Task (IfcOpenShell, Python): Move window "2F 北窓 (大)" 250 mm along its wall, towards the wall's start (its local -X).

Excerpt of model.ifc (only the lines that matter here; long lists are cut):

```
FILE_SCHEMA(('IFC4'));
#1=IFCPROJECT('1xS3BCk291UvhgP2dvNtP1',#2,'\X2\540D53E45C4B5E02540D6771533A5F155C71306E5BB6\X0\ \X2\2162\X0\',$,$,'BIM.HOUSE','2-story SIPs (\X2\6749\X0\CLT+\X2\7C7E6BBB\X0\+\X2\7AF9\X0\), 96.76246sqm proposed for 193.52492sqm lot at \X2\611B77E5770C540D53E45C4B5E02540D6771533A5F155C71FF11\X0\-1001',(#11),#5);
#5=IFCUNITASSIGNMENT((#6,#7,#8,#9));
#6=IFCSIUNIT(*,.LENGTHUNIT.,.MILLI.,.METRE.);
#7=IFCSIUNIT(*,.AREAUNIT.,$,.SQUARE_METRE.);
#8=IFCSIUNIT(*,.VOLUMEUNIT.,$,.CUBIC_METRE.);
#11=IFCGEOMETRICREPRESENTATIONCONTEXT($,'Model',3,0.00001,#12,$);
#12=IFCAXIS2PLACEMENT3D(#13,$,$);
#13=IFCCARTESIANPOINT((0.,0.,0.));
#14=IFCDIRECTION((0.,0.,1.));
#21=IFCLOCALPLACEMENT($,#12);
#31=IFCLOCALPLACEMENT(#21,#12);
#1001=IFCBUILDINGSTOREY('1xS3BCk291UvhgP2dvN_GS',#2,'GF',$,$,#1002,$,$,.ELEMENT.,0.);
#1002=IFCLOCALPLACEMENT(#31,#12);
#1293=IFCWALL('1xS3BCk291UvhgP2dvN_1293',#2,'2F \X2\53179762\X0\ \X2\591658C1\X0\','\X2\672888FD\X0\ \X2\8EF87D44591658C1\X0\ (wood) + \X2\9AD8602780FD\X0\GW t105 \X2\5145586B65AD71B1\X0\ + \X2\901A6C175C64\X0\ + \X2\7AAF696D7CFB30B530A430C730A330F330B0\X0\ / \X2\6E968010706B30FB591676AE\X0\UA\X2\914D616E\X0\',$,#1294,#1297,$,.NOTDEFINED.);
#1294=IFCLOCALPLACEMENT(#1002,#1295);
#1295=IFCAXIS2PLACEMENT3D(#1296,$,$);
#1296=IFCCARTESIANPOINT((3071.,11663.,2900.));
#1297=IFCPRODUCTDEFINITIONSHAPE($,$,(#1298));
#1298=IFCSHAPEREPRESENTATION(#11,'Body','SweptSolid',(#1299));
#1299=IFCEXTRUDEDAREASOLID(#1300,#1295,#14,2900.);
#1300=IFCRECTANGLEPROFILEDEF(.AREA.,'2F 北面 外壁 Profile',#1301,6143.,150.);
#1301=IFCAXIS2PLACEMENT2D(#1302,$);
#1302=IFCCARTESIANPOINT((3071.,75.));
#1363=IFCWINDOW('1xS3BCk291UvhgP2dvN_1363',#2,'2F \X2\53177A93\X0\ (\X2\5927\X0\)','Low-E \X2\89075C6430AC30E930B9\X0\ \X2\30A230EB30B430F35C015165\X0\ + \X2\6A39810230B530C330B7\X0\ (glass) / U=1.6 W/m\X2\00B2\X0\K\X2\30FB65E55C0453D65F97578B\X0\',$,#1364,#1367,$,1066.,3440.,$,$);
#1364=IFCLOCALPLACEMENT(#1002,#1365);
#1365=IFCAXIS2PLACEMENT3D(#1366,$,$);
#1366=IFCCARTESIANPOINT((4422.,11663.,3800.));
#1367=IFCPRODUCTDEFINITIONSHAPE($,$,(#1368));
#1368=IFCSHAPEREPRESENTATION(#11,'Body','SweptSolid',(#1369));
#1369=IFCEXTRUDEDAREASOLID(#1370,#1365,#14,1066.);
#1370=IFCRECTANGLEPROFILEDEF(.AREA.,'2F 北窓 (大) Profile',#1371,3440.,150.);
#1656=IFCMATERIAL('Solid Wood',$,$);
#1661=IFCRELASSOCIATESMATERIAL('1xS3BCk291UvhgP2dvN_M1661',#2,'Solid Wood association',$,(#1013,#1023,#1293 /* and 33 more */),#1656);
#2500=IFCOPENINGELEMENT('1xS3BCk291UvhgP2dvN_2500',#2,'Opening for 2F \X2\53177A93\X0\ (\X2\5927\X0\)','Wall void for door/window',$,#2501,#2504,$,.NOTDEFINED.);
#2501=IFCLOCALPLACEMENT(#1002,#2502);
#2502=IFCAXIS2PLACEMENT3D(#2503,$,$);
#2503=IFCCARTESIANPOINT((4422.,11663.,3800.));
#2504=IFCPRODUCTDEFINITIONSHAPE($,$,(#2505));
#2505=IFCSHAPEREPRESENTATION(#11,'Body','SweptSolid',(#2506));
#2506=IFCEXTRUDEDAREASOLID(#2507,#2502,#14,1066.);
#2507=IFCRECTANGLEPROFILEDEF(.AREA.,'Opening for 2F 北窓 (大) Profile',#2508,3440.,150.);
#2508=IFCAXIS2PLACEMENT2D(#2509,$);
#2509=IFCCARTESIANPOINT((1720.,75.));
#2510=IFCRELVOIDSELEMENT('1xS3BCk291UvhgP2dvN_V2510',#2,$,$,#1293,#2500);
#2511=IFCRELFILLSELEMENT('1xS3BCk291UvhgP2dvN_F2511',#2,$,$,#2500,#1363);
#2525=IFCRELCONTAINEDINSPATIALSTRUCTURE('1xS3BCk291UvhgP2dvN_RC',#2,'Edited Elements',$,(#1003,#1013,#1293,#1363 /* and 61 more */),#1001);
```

```python
import ifcopenshell
import ifcopenshell.api.geometry
import ifcopenshell.util.placement
import ifcopenshell.util.unit

model = ifcopenshell.open("model.ifc")
unit_scale = ifcopenshell.util.unit.calculate_unit_scale(model)

window = model.by_guid("1xS3BCk291UvhgP2dvN_1363")
opening = window.FillsVoids[0].RelatingOpeningElement
wall = opening.VoidsElements[0].RelatingBuildingElement

wall_matrix = ifcopenshell.util.placement.get_local_placement(wall.ObjectPlacement)
shift = wall_matrix[:3, 0] * -0.25 / unit_scale
before = ifcopenshell.util.placement.get_local_placement(window.ObjectPlacement)[:3, 3].copy()

# The window is not placed relative to its opening, so move both.
for product in (opening, window):
    matrix = ifcopenshell.util.placement.get_local_placement(product.ObjectPlacement)
    matrix[:3, 3] += shift
    ifcopenshell.api.geometry.edit_object_placement(model, product=product, matrix=matrix, is_si=False)

after = ifcopenshell.util.placement.get_local_placement(window.ObjectPlacement)[:3, 3]
print("window moved by", (after - before).round(3) + 0.0)

model.write("model_v2.ifc")
```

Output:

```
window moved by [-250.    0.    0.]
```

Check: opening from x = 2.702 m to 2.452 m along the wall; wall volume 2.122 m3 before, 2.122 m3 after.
